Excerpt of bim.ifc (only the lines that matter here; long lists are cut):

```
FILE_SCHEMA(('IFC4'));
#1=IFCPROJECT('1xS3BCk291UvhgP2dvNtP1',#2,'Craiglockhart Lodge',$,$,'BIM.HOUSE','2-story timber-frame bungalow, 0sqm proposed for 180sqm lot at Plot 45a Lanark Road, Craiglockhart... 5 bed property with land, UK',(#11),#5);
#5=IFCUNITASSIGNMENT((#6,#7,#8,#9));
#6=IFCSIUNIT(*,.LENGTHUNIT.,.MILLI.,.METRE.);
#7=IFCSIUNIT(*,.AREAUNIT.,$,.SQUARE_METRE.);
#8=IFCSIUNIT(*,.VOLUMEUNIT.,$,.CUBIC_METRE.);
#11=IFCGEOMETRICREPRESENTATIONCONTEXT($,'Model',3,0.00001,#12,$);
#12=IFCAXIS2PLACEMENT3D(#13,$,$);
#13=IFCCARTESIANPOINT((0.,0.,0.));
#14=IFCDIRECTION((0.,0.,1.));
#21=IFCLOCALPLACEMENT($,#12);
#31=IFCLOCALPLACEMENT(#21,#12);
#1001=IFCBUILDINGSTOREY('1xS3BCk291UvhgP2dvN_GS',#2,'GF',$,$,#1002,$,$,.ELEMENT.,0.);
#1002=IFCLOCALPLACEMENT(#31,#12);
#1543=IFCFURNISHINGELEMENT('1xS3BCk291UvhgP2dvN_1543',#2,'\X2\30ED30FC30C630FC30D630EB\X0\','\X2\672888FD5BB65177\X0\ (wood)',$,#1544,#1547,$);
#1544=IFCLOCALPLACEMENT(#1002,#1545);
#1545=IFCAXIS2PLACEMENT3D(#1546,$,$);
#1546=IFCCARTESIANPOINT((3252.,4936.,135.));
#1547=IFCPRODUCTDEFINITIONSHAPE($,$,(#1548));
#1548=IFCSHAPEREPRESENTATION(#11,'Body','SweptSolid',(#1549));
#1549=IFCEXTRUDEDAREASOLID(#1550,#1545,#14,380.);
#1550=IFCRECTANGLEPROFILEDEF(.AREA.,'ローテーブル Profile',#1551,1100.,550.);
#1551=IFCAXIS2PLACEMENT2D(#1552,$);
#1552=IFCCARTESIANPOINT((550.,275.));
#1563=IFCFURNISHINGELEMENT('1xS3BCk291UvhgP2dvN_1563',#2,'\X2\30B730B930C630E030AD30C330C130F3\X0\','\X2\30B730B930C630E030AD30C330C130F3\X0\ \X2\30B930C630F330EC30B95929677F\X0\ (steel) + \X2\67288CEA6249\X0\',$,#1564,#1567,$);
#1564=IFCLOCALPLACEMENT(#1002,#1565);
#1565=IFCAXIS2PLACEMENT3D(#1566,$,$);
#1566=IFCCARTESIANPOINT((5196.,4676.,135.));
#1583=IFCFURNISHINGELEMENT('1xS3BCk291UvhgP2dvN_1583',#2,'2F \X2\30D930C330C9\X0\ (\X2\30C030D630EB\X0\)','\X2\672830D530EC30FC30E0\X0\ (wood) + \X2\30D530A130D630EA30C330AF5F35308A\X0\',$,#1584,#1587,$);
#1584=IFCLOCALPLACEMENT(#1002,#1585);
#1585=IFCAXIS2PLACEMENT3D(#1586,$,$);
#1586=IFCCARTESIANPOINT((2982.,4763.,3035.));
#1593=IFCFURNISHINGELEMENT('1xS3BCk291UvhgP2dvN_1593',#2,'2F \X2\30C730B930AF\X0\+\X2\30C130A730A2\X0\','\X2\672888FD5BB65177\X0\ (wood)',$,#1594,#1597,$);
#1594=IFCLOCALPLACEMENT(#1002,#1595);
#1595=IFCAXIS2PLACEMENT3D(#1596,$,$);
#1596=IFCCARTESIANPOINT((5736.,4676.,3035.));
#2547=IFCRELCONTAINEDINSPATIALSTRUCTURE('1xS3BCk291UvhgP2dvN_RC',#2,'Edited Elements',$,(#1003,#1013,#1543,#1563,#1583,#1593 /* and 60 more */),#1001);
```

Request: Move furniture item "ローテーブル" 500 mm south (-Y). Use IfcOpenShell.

```python
import ifcopenshell
import ifcopenshell.api.geometry
import ifcopenshell.util.placement

model = ifcopenshell.open("bim.ifc")

item = model.by_guid("1xS3BCk291UvhgP2dvN_1543")
matrix = ifcopenshell.util.placement.get_local_placement(item.ObjectPlacement)
matrix[1, 3] -= 500.0
ifcopenshell.api.geometry.edit_object_placement(model, product=item, matrix=matrix, is_si=False)

print(ifcopenshell.util.placement.get_local_placement(item.ObjectPlacement).round(3) + 0.0)

model.write("bim_v2.ifc")
```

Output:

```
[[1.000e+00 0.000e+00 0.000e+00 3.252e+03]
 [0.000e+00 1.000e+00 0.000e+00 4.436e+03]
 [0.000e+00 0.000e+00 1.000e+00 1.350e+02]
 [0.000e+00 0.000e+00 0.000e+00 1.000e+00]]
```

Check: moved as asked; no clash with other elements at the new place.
